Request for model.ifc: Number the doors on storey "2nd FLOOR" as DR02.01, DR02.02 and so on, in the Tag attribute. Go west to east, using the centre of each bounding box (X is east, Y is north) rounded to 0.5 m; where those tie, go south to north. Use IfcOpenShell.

First a look at what the model holds.

```python
import ifcopenshell
import ifcopenshell.util.element
import ifcopenshell.util.placement

model = ifcopenshell.open("model.ifc")
print(model.schema)
storey = next(s for s in model.by_type("IfcBuildingStorey") if s.Name == "2nd FLOOR")
doors = [e for e in ifcopenshell.util.element.get_decomposition(storey) if e.is_a("IfcDoor")]
for e in sorted(doors, key=lambda e: e.id()):
    origin = ifcopenshell.util.placement.get_local_placement(e.ObjectPlacement)[:3, 3]
    print(e.id(), e.Tag, e.Name, origin.round(2) + 0.0, sep=" | ")
```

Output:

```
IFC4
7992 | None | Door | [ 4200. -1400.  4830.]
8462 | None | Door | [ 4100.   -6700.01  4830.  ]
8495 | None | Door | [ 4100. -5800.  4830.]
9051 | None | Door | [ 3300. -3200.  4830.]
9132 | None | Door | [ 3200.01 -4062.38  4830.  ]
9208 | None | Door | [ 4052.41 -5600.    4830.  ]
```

```python
import ifcopenshell
import ifcopenshell.geom
import ifcopenshell.util.element
import ifcopenshell.util.shape

model = ifcopenshell.open("model.ifc")
settings = ifcopenshell.geom.settings()
settings.set("use-world-coords", True)


def centre(element):
    shape = ifcopenshell.geom.create_shape(settings, element)
    return ifcopenshell.util.shape.get_bbox_centroid(shape.geometry)


storey = next(s for s in model.by_type("IfcBuildingStorey") if s.Name == "2nd FLOOR")
doors = [e for e in ifcopenshell.util.element.get_decomposition(storey) if e.is_a("IfcDoor")]

# Insertion points can sit at a corner or the storey origin, so sort by the geometry (in metres).
centres = {e: centre(e) for e in doors}
doors.sort(key=lambda e: (round(centres[e][0] / 0.5), centres[e][1]))

for i, e in enumerate(doors, start=1):
    number = f"DR02.{i:02d}"
    e.Tag = number
    print(e.id(), number)

model.write("model_v2.ifc")
```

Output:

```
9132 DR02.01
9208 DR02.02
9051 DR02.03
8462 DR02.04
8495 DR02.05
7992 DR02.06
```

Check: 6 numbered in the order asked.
